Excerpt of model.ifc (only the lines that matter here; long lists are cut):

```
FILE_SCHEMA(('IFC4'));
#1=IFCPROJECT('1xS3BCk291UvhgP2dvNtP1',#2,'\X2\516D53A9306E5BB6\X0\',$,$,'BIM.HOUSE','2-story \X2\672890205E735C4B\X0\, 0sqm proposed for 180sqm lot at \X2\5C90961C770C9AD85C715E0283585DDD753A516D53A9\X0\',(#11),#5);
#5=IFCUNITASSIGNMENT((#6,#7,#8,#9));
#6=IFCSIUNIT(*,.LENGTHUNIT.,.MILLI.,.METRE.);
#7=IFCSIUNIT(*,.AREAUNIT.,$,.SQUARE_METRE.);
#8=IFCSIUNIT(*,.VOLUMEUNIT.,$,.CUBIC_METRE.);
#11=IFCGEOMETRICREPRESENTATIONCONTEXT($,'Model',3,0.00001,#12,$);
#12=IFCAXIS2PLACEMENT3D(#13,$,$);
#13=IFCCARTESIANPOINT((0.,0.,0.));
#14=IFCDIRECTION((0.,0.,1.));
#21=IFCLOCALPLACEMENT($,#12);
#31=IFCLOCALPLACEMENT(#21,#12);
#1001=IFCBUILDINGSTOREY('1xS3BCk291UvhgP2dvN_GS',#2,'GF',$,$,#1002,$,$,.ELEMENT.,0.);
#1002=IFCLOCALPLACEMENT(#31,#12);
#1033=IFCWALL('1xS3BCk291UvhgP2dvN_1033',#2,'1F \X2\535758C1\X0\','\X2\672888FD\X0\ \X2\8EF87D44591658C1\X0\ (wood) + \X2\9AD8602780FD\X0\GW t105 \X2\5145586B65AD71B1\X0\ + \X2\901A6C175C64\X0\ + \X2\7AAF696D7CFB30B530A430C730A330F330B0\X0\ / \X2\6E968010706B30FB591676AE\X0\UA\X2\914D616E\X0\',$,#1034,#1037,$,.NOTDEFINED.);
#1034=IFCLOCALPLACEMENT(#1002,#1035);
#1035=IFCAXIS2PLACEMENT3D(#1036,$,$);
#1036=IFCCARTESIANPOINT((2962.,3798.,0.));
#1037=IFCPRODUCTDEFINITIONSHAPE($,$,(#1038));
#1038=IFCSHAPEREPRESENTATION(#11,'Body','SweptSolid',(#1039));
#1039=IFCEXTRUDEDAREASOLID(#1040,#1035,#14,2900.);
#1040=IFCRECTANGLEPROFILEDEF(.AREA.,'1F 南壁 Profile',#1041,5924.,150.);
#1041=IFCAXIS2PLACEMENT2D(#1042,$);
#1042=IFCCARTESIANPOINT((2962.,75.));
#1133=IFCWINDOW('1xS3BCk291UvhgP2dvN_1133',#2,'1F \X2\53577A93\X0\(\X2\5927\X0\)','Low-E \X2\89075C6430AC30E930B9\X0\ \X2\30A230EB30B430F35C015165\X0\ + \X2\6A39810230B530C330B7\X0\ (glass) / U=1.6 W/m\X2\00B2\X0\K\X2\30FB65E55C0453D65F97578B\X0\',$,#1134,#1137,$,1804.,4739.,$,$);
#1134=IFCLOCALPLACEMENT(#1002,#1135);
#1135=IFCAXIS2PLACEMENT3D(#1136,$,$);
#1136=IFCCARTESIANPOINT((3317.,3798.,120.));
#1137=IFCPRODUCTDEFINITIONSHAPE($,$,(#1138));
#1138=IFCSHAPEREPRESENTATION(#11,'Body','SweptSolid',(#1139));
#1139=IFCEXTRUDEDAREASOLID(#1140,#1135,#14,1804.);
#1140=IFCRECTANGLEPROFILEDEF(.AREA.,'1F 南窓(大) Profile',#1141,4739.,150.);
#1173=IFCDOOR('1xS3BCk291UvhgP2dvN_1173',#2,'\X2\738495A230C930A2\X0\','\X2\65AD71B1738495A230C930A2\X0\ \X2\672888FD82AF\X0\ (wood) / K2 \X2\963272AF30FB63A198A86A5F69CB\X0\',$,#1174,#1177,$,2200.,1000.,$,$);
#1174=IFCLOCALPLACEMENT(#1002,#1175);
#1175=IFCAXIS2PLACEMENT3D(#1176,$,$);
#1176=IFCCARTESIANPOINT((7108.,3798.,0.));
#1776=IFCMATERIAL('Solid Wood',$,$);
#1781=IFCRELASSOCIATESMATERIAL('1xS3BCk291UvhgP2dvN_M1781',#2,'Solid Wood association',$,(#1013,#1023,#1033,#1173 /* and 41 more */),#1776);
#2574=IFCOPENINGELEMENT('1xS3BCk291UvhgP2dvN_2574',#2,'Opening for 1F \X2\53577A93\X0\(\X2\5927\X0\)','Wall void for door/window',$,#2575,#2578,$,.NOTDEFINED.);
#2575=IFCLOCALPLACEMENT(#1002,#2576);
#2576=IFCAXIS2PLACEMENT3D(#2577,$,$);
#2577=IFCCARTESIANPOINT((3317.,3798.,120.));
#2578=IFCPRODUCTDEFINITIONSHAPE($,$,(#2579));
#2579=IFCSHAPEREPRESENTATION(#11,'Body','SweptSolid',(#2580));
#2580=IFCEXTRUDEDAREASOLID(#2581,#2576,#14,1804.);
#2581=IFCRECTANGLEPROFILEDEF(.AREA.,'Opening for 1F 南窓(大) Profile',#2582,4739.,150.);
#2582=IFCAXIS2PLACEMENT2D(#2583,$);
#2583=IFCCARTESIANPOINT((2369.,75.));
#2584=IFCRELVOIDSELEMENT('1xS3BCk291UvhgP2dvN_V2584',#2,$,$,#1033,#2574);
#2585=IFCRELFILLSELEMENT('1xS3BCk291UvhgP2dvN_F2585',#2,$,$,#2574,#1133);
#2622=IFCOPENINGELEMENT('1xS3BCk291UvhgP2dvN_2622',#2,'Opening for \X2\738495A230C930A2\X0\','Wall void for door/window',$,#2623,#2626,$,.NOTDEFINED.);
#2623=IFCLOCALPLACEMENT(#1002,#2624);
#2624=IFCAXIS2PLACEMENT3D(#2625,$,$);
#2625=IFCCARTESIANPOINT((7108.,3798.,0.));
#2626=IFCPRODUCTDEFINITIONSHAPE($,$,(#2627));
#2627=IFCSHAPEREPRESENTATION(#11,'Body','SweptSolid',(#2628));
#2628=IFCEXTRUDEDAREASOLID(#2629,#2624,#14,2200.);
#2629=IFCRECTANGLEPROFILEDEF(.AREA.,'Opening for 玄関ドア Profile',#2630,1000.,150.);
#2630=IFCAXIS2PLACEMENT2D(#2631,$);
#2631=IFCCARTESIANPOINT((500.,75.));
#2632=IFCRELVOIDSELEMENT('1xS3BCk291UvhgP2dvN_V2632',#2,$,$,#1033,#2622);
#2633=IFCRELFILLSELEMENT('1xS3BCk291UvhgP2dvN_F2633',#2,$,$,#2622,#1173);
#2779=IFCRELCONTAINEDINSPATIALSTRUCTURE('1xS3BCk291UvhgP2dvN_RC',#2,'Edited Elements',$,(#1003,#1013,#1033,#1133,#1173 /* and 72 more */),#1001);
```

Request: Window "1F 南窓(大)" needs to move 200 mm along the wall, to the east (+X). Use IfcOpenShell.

```python
import ifcopenshell
import ifcopenshell.api.geometry
import ifcopenshell.util.placement

model = ifcopenshell.open("model.ifc")

window = model.by_guid("1xS3BCk291UvhgP2dvN_1133")
opening = window.FillsVoids[0].RelatingOpeningElement
wall = opening.VoidsElements[0].RelatingBuildingElement

wall_matrix = ifcopenshell.util.placement.get_local_placement(wall.ObjectPlacement)
shift = wall_matrix[:3, 0] * 200.0
before = ifcopenshell.util.placement.get_local_placement(window.ObjectPlacement)[:3, 3].copy()

# The window is not placed relative to its opening, so move both.
for product in (opening, window):
    matrix = ifcopenshell.util.placement.get_local_placement(product.ObjectPlacement)
    matrix[:3, 3] += shift
    ifcopenshell.api.geometry.edit_object_placement(model, product=product, matrix=matrix, is_si=False)

after = ifcopenshell.util.placement.get_local_placement(window.ObjectPlacement)[:3, 3]
print("window moved by", (after - before).round(3) + 0.0)

model.write("model_v2.ifc")
```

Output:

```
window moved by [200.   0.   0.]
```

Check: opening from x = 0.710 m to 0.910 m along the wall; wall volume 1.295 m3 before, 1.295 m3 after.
